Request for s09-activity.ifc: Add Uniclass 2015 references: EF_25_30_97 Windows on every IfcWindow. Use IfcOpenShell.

First a look at what the model holds.

```python
import ifcopenshell

model = ifcopenshell.open("s09-activity.ifc")
print(model.schema)
print("classifications:", [c.Name for c in model.by_type("IfcClassification")])
for ifc_class in ("IfcDoor", "IfcRoof", "IfcStair", "IfcWall", "IfcWindow"):
    print(ifc_class, len(model.by_type(ifc_class)))
```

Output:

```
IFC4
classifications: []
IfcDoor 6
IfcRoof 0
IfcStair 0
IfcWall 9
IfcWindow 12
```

```python
import ifcopenshell
import ifcopenshell.api.classification

model = ifcopenshell.open("s09-activity.ifc")

system = ifcopenshell.api.classification.add_classification(model, classification="Uniclass 2015")

codes = {
    "IfcWindow": ("EF_25_30_97", "Windows"),
}
for ifc_class, (code, name) in codes.items():
    products = model.by_type(ifc_class)
    ifcopenshell.api.classification.add_reference(
        model, products=products, classification=system, identification=code, name=name
    )
    print(code, len(products))

model.write("s09-activity_rev.ifc")
```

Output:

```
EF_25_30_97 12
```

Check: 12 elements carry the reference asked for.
